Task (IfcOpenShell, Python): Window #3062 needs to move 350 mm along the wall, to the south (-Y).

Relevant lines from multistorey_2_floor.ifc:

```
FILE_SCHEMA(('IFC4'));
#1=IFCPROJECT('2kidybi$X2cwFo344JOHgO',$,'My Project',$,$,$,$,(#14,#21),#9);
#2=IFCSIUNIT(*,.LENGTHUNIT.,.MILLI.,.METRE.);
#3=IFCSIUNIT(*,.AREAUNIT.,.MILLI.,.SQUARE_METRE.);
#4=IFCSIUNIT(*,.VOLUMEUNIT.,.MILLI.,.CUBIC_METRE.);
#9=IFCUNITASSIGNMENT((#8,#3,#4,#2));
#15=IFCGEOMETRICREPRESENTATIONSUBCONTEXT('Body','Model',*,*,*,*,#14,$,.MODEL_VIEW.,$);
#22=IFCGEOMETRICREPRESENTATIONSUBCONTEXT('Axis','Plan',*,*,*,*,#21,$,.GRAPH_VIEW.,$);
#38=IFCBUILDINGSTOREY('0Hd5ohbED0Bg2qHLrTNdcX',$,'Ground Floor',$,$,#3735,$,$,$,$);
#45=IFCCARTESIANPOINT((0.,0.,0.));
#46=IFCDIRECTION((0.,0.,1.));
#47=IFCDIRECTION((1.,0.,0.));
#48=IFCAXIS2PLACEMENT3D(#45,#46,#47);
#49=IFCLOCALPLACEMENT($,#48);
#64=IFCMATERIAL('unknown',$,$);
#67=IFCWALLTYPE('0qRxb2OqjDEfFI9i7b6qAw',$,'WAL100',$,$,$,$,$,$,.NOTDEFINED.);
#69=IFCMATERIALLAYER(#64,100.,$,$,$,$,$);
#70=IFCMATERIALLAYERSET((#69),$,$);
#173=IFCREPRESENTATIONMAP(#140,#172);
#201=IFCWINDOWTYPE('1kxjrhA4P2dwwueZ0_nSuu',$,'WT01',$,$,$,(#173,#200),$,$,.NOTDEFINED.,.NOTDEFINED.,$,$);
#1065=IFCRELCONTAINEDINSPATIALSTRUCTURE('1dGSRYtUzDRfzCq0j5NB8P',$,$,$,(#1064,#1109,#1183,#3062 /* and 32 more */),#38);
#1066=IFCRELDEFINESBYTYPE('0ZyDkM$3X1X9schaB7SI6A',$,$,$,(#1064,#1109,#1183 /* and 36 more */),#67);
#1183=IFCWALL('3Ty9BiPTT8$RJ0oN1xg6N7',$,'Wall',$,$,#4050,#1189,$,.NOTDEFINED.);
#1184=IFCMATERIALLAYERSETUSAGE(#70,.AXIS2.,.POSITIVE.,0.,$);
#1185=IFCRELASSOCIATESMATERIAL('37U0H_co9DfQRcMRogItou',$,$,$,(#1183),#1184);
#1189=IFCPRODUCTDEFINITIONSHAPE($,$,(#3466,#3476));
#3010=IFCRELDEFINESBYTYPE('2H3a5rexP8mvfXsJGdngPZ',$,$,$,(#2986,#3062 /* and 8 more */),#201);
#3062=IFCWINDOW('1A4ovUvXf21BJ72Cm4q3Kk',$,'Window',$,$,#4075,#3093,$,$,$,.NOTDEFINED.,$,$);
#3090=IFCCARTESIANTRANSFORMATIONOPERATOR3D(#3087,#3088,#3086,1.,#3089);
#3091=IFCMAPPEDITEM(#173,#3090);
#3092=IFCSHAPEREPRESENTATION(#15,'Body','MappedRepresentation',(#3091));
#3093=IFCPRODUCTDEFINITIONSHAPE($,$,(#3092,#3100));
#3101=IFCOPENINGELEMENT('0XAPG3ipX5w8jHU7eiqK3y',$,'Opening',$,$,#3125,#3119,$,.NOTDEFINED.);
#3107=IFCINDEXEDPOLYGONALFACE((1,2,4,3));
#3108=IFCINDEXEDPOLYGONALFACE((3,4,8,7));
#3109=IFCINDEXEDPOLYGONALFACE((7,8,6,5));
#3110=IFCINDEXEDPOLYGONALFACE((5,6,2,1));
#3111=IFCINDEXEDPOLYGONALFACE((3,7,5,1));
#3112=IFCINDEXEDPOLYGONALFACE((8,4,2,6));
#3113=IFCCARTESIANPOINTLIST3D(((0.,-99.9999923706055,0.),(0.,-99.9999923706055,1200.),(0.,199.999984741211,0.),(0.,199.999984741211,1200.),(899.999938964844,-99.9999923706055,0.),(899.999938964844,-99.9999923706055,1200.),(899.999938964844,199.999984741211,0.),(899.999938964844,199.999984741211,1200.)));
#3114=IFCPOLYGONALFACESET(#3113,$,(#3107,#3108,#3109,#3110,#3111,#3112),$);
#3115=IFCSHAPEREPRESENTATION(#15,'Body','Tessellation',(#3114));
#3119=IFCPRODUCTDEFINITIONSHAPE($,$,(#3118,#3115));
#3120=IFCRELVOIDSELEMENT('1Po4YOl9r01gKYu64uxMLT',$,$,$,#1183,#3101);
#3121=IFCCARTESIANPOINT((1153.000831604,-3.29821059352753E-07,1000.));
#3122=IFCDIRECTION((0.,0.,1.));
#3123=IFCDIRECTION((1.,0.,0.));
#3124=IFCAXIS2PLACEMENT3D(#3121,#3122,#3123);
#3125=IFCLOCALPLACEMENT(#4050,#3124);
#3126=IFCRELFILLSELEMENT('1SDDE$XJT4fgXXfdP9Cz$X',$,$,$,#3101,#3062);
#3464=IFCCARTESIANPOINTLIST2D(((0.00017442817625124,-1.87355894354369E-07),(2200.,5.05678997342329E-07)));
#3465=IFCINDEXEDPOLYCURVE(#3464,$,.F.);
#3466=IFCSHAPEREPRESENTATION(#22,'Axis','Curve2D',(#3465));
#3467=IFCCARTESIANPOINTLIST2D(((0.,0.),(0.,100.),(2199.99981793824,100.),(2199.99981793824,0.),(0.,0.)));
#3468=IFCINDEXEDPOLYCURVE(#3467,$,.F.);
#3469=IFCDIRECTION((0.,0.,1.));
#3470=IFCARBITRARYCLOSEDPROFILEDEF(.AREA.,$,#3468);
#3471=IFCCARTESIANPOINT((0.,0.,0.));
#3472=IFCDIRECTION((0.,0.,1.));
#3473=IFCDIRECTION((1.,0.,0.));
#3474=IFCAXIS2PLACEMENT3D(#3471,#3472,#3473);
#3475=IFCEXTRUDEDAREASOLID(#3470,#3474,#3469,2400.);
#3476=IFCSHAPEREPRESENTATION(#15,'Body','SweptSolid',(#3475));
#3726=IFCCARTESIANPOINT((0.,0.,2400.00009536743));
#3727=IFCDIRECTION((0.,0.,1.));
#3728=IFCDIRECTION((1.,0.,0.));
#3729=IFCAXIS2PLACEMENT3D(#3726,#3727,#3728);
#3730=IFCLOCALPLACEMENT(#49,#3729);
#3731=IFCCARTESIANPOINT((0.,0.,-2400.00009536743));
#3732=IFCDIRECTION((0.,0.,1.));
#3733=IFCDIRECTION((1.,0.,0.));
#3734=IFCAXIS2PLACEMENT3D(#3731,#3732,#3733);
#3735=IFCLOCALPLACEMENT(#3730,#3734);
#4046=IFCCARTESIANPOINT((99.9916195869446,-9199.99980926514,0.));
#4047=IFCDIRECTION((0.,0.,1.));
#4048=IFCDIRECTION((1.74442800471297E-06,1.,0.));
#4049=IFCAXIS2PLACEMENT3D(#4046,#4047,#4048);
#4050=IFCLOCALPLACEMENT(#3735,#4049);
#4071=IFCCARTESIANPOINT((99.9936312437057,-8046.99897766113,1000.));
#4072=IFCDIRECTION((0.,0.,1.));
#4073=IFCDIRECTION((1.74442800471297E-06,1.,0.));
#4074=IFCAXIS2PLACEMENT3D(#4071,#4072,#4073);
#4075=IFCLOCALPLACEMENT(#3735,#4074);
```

```python
import ifcopenshell
import ifcopenshell.api.geometry
import ifcopenshell.util.placement
import ifcopenshell.util.unit

model = ifcopenshell.open("multistorey_2_floor.ifc")
unit_scale = ifcopenshell.util.unit.calculate_unit_scale(model)

window = model.by_guid("1A4ovUvXf21BJ72Cm4q3Kk")
opening = window.FillsVoids[0].RelatingOpeningElement
wall = opening.VoidsElements[0].RelatingBuildingElement

wall_matrix = ifcopenshell.util.placement.get_local_placement(wall.ObjectPlacement)
shift = wall_matrix[:3, 0] * -0.35 / unit_scale
before = ifcopenshell.util.placement.get_local_placement(window.ObjectPlacement)[:3, 3].copy()

# The window is not placed relative to its opening, so move both.
for product in (opening, window):
    matrix = ifcopenshell.util.placement.get_local_placement(product.ObjectPlacement)
    matrix[:3, 3] += shift
    ifcopenshell.api.geometry.edit_object_placement(model, product=product, matrix=matrix, is_si=False)

after = ifcopenshell.util.placement.get_local_placement(window.ObjectPlacement)[:3, 3]
print("window moved by", (after - before).round(3) + 0.0)

model.write("multistorey_2_floor_edited.ifc")
```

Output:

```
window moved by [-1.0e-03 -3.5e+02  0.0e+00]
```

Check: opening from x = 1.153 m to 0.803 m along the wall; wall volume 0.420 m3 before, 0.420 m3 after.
